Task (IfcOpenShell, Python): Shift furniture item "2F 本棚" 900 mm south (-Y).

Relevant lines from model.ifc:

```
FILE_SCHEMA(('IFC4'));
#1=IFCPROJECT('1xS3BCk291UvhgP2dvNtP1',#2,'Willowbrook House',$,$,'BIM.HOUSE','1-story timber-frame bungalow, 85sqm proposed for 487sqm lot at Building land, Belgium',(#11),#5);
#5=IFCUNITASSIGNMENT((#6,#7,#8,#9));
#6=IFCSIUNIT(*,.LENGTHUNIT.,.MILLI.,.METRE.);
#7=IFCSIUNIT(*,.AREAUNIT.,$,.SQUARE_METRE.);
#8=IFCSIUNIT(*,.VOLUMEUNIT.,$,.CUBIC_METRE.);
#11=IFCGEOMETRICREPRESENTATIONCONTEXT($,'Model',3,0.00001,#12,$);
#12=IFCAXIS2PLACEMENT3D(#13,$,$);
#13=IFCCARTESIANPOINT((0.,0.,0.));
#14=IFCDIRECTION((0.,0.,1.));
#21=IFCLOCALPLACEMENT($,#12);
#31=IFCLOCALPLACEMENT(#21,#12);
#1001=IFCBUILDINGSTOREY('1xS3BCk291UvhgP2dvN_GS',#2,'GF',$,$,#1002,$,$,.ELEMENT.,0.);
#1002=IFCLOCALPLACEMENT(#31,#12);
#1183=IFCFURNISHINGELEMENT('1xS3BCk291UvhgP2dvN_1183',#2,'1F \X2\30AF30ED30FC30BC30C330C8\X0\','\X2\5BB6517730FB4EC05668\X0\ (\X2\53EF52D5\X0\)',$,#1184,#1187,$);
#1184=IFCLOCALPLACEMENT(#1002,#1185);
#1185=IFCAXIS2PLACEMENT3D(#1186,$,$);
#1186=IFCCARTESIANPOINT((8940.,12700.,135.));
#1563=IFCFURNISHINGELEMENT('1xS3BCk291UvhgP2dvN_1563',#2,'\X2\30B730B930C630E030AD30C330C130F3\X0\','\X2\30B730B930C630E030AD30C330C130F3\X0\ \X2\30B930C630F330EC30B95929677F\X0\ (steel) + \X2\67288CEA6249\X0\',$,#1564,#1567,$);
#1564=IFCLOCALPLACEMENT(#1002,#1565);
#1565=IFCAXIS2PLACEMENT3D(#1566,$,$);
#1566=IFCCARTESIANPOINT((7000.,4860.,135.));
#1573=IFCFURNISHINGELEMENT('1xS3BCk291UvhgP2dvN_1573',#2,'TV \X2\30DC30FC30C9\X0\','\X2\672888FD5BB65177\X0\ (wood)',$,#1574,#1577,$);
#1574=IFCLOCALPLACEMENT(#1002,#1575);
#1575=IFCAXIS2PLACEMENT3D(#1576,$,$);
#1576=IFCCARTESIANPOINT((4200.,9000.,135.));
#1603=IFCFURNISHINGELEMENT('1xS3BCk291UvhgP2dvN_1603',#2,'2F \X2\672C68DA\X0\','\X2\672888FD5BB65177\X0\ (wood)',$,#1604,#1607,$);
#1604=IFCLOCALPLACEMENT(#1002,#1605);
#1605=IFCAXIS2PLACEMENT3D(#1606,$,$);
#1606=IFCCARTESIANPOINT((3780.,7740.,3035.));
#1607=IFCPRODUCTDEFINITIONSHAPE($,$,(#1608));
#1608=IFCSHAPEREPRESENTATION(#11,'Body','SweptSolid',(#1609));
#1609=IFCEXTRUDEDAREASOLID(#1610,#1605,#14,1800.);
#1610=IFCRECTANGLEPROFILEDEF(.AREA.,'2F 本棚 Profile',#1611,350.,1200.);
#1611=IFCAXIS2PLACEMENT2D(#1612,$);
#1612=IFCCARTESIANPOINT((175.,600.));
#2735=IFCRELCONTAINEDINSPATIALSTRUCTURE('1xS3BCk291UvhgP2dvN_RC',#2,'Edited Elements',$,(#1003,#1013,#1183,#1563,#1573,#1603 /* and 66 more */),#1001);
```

```python
import ifcopenshell
import ifcopenshell.api.geometry
import ifcopenshell.util.placement

model = ifcopenshell.open("model.ifc")

item = model.by_guid("1xS3BCk291UvhgP2dvN_1603")
matrix = ifcopenshell.util.placement.get_local_placement(item.ObjectPlacement)
matrix[1, 3] -= 900.0
ifcopenshell.api.geometry.edit_object_placement(model, product=item, matrix=matrix, is_si=False)

print(ifcopenshell.util.placement.get_local_placement(item.ObjectPlacement).round(3) + 0.0)

model.write("model-out.ifc")
```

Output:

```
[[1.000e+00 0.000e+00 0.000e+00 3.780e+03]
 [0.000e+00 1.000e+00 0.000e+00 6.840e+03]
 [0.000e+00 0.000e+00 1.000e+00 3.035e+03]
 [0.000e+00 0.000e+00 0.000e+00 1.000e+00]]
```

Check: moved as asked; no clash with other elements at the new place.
